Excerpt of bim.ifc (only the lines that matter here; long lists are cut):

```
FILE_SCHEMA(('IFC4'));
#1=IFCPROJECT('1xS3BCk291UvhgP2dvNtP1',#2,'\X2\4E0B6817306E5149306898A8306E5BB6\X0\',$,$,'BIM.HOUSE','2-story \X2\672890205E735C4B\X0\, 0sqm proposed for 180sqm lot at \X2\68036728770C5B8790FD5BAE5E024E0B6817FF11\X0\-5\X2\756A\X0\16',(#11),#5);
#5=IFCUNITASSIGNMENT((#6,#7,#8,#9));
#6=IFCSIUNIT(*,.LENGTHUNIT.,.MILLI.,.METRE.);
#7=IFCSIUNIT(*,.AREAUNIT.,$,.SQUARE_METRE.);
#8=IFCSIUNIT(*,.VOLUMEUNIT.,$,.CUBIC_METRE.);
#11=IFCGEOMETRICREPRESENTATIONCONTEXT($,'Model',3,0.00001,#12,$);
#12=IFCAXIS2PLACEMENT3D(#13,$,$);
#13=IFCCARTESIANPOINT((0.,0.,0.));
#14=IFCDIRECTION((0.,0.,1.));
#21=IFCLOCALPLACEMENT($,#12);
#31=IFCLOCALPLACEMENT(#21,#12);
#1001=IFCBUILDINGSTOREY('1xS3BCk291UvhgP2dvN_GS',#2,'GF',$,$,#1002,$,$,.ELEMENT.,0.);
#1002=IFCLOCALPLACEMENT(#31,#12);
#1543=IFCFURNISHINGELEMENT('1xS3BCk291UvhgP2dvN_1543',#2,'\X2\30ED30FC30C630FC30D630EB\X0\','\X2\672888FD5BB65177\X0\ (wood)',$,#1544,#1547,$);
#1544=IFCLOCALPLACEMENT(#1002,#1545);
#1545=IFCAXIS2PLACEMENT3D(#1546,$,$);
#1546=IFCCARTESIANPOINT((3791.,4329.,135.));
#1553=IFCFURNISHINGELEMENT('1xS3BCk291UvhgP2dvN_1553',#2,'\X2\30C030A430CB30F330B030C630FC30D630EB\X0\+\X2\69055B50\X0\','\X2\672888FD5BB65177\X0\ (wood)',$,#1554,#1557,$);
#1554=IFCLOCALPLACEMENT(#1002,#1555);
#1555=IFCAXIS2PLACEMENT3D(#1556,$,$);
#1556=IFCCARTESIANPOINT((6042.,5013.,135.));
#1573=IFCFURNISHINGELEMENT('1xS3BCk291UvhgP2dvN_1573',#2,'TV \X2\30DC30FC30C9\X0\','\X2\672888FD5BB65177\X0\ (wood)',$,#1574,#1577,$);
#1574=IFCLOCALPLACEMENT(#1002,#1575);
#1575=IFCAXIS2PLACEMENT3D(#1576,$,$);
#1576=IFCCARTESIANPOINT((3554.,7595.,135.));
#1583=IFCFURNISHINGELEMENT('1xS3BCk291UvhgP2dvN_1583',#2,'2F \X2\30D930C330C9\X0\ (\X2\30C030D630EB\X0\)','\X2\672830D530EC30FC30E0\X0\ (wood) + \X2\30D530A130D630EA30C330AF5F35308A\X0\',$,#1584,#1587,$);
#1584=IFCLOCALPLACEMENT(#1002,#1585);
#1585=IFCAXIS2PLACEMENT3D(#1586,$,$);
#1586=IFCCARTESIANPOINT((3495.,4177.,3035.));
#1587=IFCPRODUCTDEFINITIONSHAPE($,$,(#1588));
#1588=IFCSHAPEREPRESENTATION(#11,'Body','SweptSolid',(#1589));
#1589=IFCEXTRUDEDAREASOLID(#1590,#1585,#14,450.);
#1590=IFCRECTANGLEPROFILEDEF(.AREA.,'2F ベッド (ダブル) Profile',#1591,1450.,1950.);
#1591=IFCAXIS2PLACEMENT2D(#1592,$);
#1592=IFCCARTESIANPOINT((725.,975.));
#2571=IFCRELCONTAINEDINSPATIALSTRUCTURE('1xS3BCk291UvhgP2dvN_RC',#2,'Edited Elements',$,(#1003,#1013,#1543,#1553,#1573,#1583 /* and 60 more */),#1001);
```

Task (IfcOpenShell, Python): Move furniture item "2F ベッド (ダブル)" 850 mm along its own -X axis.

```python
import ifcopenshell
import ifcopenshell.api.geometry
import ifcopenshell.util.placement
import ifcopenshell.util.unit

model = ifcopenshell.open("bim.ifc")
unit_scale = ifcopenshell.util.unit.calculate_unit_scale(model)

item = model.by_guid("1xS3BCk291UvhgP2dvN_1583")
matrix = ifcopenshell.util.placement.get_local_placement(item.ObjectPlacement)
matrix[:3, 3] -= matrix[:3, 0] * 0.85 / unit_scale
ifcopenshell.api.geometry.edit_object_placement(model, product=item, matrix=matrix, is_si=False)

print(ifcopenshell.util.placement.get_local_placement(item.ObjectPlacement).round(3) + 0.0)

model.write("bim_v2.ifc")
```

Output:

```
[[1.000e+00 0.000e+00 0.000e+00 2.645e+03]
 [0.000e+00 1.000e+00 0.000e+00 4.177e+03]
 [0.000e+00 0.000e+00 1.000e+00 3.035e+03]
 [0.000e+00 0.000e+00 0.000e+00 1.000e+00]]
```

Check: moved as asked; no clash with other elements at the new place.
